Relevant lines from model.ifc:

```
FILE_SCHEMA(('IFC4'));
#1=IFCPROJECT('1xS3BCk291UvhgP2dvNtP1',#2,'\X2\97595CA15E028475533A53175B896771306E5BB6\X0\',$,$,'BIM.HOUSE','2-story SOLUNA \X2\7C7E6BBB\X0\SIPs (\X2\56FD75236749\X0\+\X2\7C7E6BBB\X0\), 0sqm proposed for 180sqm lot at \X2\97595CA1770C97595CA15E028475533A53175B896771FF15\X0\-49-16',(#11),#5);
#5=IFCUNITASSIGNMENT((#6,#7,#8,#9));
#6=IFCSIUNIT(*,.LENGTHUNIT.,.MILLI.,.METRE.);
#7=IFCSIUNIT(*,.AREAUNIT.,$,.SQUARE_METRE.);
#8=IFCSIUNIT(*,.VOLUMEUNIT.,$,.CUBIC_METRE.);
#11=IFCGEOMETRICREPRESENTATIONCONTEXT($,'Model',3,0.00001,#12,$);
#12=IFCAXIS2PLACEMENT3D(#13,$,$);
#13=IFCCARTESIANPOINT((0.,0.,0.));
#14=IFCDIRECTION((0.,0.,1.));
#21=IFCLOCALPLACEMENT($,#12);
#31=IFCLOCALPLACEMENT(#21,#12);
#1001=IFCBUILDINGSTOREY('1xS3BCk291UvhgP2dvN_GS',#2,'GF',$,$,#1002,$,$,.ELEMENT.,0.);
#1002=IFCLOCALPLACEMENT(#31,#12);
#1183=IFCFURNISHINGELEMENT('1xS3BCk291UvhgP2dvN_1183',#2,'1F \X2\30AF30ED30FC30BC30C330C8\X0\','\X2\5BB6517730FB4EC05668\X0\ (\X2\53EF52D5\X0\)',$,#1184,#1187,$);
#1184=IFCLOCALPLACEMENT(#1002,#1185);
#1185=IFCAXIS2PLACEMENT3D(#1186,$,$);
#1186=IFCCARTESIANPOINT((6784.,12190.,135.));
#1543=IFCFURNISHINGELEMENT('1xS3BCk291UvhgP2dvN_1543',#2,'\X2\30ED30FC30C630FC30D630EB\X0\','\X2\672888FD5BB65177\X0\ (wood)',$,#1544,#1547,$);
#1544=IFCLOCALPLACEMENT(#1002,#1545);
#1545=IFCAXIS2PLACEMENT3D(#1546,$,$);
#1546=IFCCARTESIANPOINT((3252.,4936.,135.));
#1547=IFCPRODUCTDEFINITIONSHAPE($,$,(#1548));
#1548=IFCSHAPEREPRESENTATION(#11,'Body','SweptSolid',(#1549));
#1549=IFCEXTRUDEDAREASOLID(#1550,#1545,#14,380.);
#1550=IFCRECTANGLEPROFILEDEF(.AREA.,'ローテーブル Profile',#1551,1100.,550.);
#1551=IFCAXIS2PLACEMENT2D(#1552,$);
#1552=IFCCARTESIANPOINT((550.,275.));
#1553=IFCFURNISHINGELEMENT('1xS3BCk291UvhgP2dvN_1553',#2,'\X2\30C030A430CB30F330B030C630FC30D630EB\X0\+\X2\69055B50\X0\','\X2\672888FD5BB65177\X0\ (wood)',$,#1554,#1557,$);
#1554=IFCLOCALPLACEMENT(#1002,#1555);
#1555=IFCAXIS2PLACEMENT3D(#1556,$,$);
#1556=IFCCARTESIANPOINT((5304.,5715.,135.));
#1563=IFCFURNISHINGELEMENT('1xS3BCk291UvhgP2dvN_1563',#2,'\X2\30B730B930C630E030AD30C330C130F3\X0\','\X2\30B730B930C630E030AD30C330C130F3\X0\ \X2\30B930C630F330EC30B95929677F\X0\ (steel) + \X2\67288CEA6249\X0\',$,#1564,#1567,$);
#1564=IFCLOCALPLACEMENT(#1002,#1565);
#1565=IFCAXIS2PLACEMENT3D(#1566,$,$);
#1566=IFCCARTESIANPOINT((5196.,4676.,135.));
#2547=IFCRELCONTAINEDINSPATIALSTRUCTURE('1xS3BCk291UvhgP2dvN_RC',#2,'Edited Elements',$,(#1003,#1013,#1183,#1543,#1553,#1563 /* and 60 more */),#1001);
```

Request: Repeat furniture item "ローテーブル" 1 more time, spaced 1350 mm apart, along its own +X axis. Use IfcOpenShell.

```python
import ifcopenshell
import ifcopenshell.api.geometry
import ifcopenshell.api.root
import ifcopenshell.util.element
import ifcopenshell.util.placement
import ifcopenshell.util.unit

model = ifcopenshell.open("model.ifc")
unit_scale = ifcopenshell.util.unit.calculate_unit_scale(model)


def reuse_history(source, copy):
    """copy_class also copies each property set's owner history, people and application; keep the originals."""
    for rel in copy.IsDefinedBy:
        if rel.is_a("IfcRelDefinesByProperties") and (history := rel.RelatingPropertyDefinition.OwnerHistory):
            rel.RelatingPropertyDefinition.OwnerHistory = source.OwnerHistory
            ifcopenshell.util.element.remove_deep2(model, history)


source = model.by_guid("1xS3BCk291UvhgP2dvN_1543")
base = ifcopenshell.util.placement.get_local_placement(source.ObjectPlacement)
step = base[:3, 0] * 1.35 / unit_scale

for i in range(1, 2):
    copy = ifcopenshell.api.root.copy_class(model, product=source)
    copy.Representation = ifcopenshell.util.element.copy_deep(
        model, source.Representation, exclude=["IfcGeometricRepresentationContext", "IfcRepresentationMap"]
    )
    reuse_history(source, copy)
    matrix = base.copy()
    matrix[:3, 3] += i * step
    print("added at", matrix[:3, 3].round(3) + 0.0)
    ifcopenshell.api.geometry.edit_object_placement(model, product=copy, matrix=matrix, is_si=False)

model.write("model_rev.ifc")
```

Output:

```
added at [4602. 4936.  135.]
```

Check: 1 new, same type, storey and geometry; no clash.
